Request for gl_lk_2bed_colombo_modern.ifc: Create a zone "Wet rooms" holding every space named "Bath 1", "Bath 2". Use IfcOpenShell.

First a look at what the model holds.

```python
import ifcopenshell

model = ifcopenshell.open("gl_lk_2bed_colombo_modern.ifc")
print(model.schema)
seen = {}
for space in model.by_type("IfcSpace"):
    seen[space.LongName] = seen.get(space.LongName, 0) + 1
for name, count in sorted(seen.items(), key=str):
    print(count, "x", name)
print("zones:", [z.Name for z in model.by_type("IfcZone")][:20])
```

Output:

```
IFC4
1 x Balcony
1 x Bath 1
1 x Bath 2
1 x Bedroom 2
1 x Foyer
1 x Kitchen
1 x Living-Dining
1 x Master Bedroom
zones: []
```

```python
import ifcopenshell
import ifcopenshell.api.group
import ifcopenshell.api.root

model = ifcopenshell.open("gl_lk_2bed_colombo_modern.ifc")

names = {"Bath 1", "Bath 2"}
spaces = [s for s in model.by_type("IfcSpace") if s.LongName in names]

zone = ifcopenshell.api.root.create_entity(model, ifc_class="IfcZone", name="Wet rooms")
ifcopenshell.api.group.assign_group(model, products=spaces, group=zone)
print(len(spaces), "spaces in", zone.Name)

model.write("gl_lk_2bed_colombo_modern_edited.ifc")
```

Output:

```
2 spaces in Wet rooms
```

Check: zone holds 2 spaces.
